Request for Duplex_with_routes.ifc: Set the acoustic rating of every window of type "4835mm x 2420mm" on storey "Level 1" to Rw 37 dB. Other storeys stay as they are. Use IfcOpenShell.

First a look at what the model holds.

```python
import ifcopenshell
import ifcopenshell.util.element

model = ifcopenshell.open("Duplex_with_routes.ifc")
print(model.schema)
storey = next(s for s in model.by_type("IfcBuildingStorey") if s.Name == "Level 1")
windows = [e for e in ifcopenshell.util.element.get_decomposition(storey) if e.is_a("IfcWindow")]
seen = {}
for e in windows:
    element_type = ifcopenshell.util.element.get_type(e)
    key = (element_type.Name if element_type != e and element_type else None, ifcopenshell.util.element.get_pset(e, "Pset_WindowCommon", "AcousticRating"))
    seen[key] = seen.get(key, 0) + 1
for (name, value), count in sorted(seen.items(), key=str):
    print(count, "x", name, "|", value)
```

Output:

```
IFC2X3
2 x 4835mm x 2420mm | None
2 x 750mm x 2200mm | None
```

```python
import ifcopenshell
import ifcopenshell.api.pset
import ifcopenshell.util.element

model = ifcopenshell.open("Duplex_with_routes.ifc")

storey = next(s for s in model.by_type("IfcBuildingStorey") if s.Name == "Level 1")
windows = [e for e in ifcopenshell.util.element.get_decomposition(storey) if e.is_a("IfcWindow")]

count = 0
for e in windows:
    element_type = ifcopenshell.util.element.get_type(e)
    if element_type in (None, e) or element_type.Name != "4835mm x 2420mm":
        continue
    # add_pset returns the element's existing set when there is one.
    pset = ifcopenshell.api.pset.add_pset(model, product=e, name="Pset_WindowCommon")
    ifcopenshell.api.pset.edit_pset(model, pset=pset, properties={"AcousticRating": "Rw 37 dB"})
    count += 1

print(count, "windows updated")

model.write("Duplex_with_routes_rev.ifc")
```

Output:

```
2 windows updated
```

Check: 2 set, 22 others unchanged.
